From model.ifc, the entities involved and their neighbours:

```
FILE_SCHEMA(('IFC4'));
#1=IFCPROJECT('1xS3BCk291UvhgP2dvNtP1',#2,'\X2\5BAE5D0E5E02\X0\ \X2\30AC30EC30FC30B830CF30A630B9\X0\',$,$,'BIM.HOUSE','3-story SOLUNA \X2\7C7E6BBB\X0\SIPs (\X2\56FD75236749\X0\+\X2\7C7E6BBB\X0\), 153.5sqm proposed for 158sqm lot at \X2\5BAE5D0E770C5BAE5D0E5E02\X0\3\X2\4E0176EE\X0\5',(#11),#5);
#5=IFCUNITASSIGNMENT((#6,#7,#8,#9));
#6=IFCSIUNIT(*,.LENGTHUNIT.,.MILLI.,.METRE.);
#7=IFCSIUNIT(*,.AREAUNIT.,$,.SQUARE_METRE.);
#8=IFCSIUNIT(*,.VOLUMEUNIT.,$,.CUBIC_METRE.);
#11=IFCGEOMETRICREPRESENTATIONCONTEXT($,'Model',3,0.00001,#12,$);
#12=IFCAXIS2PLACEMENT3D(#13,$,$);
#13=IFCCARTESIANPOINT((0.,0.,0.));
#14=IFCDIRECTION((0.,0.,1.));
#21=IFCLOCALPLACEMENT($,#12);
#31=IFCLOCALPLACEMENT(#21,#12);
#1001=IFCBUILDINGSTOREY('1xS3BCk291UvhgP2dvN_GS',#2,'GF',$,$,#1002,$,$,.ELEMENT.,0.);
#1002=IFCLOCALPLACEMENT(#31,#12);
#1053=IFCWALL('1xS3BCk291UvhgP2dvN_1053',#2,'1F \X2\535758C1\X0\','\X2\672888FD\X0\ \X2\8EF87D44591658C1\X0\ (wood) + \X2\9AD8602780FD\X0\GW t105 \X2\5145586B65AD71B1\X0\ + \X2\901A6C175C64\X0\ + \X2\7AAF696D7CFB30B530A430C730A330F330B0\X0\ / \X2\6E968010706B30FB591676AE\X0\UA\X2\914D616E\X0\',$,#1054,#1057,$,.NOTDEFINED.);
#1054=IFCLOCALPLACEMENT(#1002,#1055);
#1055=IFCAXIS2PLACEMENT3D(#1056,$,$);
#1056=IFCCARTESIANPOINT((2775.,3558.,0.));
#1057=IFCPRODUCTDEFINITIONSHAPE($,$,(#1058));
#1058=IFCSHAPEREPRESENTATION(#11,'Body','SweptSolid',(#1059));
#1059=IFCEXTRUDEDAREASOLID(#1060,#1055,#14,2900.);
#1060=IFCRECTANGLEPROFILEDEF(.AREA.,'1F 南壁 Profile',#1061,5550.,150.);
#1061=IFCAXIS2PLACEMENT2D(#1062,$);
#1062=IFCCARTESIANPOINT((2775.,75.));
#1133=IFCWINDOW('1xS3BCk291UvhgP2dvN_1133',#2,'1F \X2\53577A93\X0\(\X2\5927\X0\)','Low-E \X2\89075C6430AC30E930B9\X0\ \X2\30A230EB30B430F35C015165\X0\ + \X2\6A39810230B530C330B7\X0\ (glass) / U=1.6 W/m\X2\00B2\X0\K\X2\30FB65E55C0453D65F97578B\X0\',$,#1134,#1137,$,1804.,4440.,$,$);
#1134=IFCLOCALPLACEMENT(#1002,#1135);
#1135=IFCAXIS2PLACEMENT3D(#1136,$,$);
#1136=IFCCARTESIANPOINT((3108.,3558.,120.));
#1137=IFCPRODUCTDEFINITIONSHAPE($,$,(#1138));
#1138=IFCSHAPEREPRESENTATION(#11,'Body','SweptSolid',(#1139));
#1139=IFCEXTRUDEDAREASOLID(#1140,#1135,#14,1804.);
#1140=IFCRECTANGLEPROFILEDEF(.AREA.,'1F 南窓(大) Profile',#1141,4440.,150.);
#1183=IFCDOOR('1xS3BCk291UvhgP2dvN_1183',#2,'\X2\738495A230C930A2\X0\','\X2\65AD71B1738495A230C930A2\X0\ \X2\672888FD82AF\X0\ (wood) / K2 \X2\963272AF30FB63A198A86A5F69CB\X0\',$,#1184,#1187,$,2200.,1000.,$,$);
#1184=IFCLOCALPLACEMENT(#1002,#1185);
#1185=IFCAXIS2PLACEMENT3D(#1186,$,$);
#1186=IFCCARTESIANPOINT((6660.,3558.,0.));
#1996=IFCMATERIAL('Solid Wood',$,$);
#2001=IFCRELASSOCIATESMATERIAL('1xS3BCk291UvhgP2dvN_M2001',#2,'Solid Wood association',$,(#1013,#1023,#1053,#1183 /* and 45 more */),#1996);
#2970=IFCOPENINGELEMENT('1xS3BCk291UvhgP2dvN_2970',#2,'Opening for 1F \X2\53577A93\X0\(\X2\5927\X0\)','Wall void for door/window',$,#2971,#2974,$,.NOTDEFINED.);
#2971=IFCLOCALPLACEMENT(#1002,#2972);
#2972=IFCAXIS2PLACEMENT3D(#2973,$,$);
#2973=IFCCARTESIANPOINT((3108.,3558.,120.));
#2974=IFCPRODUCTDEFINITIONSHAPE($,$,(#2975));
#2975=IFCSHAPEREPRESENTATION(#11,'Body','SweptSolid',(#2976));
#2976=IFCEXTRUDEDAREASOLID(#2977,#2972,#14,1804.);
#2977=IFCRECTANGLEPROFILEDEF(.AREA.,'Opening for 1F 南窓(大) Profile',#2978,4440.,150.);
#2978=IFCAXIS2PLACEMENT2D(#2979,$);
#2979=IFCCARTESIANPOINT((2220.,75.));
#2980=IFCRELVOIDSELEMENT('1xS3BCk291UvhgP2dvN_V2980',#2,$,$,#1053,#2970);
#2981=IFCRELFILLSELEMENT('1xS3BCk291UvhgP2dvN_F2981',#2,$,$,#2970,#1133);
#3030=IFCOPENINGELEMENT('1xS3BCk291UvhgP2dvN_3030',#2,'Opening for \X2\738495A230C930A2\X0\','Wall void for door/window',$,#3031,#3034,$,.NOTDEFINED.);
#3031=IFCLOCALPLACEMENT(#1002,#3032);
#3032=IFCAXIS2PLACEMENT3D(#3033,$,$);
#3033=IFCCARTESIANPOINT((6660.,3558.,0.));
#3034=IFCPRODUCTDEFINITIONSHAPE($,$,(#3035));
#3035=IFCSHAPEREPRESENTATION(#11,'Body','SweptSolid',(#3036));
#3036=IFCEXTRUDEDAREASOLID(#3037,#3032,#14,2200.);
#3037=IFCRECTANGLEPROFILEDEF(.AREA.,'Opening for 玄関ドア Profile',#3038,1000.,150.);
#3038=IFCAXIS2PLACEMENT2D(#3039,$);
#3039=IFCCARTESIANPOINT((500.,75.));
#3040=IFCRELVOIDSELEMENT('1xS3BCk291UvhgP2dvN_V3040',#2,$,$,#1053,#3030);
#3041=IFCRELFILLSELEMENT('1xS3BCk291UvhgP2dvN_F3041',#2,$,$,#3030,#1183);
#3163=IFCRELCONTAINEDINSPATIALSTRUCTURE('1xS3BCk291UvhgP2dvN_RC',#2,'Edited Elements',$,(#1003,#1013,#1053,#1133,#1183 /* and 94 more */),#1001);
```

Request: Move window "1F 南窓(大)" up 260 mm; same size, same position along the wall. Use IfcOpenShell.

```python
import numpy as np
import ifcopenshell
import ifcopenshell.api.geometry
import ifcopenshell.util.placement
import ifcopenshell.util.unit

model = ifcopenshell.open("model.ifc")
unit_scale = ifcopenshell.util.unit.calculate_unit_scale(model)

window = model.by_guid("1xS3BCk291UvhgP2dvN_1133")
opening = window.FillsVoids[0].RelatingOpeningElement
dz = 260.0

shift = np.array([0.0, 0.0, dz])
# The window is not placed relative to its opening, so move both.
for product in (opening, window):
    matrix = ifcopenshell.util.placement.get_local_placement(product.ObjectPlacement)
    matrix[:3, 3] += shift
    ifcopenshell.api.geometry.edit_object_placement(model, product=product, matrix=matrix, is_si=False)

print(f"moved by {dz * unit_scale:+.3f} m")

model.write("model_v2.ifc")
```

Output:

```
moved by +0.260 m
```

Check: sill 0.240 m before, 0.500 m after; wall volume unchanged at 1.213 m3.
